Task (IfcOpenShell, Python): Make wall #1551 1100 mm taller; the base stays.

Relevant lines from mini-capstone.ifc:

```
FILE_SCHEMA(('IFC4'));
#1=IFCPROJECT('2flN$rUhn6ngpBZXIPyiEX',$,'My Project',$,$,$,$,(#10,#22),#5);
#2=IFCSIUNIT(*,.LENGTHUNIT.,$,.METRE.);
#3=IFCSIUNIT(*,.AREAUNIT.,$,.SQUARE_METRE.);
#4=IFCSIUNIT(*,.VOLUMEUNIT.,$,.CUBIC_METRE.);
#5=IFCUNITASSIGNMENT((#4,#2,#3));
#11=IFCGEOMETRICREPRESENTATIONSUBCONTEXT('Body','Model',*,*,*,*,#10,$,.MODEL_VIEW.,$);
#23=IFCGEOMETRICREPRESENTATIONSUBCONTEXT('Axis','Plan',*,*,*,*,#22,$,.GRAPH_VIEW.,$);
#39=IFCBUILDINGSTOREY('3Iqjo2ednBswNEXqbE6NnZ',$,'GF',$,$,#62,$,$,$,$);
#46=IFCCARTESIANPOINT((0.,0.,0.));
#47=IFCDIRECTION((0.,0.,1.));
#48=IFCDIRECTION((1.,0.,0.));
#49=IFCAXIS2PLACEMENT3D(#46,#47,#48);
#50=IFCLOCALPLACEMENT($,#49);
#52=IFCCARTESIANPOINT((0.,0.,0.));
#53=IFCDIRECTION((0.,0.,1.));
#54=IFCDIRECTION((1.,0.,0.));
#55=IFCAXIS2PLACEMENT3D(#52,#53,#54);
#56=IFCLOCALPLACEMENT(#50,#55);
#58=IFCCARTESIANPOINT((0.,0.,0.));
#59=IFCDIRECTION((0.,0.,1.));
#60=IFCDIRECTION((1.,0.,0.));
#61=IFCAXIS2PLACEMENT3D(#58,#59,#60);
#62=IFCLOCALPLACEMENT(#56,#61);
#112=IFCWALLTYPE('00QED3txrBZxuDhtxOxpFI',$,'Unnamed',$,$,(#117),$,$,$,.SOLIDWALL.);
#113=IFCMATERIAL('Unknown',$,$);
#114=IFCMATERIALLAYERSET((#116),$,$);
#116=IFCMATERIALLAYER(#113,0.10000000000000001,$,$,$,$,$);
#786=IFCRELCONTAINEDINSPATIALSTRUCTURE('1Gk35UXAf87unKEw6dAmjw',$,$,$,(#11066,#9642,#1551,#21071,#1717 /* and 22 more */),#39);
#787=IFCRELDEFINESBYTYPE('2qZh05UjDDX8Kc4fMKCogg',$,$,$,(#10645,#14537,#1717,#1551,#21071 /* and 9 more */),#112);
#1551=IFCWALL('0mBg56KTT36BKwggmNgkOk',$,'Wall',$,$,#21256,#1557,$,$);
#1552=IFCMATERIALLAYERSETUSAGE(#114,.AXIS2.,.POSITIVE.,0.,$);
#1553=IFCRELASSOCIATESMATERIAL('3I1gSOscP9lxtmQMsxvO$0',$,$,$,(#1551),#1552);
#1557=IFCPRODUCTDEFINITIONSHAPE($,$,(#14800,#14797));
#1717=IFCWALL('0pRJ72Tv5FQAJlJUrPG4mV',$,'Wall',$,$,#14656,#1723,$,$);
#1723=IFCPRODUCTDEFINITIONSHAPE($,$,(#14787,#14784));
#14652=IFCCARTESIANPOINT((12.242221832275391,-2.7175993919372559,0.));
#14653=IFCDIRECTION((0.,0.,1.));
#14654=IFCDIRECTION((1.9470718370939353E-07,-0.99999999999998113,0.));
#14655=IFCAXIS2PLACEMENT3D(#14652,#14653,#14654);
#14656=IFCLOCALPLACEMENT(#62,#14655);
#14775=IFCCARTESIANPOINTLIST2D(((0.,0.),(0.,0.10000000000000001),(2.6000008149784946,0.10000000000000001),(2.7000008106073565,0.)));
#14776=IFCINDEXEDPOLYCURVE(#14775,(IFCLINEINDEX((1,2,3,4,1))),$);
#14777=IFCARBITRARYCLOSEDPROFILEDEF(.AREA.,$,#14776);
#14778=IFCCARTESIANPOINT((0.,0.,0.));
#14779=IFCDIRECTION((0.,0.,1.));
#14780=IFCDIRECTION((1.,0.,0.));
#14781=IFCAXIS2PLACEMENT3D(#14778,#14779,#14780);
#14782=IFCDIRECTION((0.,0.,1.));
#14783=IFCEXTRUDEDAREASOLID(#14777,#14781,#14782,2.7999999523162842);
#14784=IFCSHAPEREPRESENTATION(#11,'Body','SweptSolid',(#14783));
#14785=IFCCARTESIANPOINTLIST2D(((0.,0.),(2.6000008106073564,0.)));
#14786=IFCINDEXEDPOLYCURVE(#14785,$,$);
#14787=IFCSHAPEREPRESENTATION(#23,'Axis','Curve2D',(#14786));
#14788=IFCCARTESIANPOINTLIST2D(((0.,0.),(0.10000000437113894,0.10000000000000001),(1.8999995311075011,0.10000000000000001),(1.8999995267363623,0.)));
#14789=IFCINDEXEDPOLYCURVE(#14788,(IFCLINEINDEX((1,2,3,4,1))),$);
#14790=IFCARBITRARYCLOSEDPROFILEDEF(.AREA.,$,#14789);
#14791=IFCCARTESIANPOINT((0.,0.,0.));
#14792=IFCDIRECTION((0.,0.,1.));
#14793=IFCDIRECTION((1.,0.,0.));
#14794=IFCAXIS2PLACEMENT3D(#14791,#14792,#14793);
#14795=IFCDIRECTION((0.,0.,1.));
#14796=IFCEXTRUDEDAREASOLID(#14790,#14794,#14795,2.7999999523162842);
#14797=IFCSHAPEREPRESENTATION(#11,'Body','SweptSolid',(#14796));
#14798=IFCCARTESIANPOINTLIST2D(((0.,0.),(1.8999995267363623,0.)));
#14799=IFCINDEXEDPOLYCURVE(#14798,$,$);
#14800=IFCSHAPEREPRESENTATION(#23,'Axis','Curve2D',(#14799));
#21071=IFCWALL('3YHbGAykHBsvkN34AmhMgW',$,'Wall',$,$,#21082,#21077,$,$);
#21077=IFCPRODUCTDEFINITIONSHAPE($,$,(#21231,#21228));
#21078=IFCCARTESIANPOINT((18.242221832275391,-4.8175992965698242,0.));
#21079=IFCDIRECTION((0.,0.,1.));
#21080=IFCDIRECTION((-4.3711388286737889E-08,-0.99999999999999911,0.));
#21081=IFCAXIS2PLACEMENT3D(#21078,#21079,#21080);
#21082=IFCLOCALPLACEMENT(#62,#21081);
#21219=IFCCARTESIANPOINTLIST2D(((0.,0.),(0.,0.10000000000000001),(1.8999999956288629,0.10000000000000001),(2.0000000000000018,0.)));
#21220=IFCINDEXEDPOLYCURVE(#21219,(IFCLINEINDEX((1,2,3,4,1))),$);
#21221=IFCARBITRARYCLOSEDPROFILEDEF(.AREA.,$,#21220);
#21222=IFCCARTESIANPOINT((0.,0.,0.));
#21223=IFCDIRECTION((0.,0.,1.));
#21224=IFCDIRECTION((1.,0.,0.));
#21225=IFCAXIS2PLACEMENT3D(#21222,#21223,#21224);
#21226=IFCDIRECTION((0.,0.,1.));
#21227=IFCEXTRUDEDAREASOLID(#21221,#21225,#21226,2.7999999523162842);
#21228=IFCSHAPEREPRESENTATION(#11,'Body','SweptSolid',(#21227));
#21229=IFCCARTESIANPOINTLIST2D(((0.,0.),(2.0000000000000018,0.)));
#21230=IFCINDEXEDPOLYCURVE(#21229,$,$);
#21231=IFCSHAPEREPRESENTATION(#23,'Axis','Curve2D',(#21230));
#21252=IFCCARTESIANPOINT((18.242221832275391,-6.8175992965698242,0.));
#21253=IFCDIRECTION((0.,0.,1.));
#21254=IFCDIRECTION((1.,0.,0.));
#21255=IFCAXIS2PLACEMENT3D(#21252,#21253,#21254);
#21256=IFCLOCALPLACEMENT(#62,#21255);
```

```python
import ifcopenshell
import ifcopenshell.geom
import ifcopenshell.util.representation
import ifcopenshell.util.shape
import ifcopenshell.util.unit

model = ifcopenshell.open("mini-capstone.ifc")
unit_scale = ifcopenshell.util.unit.calculate_unit_scale(model)
settings = ifcopenshell.geom.settings()


def volume(element):
    """Net volume in cubic metres, openings subtracted."""
    shape = ifcopenshell.geom.create_shape(settings, element)
    return ifcopenshell.util.shape.get_volume(shape.geometry)


wall = model.by_guid("0mBg56KTT36BKwggmNgkOk")
before = volume(wall)

body = ifcopenshell.util.representation.get_representation(wall, "Model", "Body")
solid = body.Items[0]
old_height = solid.Depth
solid.Depth += 1.1 / unit_scale
after = volume(wall)

print(f"height {old_height:g} -> {solid.Depth:g}, volume {before:.3f} -> {after:.3f} m3")

model.write("mini-capstone_v2.ifc")
```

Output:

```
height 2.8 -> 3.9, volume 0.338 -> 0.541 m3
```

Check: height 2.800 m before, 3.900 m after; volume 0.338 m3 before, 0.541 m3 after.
